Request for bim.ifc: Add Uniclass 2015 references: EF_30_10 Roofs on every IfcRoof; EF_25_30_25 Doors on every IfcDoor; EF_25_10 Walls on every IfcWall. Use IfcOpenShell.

First a look at what the model holds.

```python
import ifcopenshell

model = ifcopenshell.open("bim.ifc")
print(model.schema)
print("classifications:", [c.Name for c in model.by_type("IfcClassification")])
for ifc_class in ("IfcDoor", "IfcRoof", "IfcStair", "IfcWall", "IfcWindow"):
    print(ifc_class, len(model.by_type(ifc_class)))
```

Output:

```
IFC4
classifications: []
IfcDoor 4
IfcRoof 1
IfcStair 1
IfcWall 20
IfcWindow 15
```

```python
import ifcopenshell
import ifcopenshell.api.classification

model = ifcopenshell.open("bim.ifc")

system = ifcopenshell.api.classification.add_classification(model, classification="Uniclass 2015")

codes = {
    "IfcRoof": ("EF_30_10", "Roofs"),
    "IfcDoor": ("EF_25_30_25", "Doors"),
    "IfcWall": ("EF_25_10", "Walls"),
}
for ifc_class, (code, name) in codes.items():
    products = model.by_type(ifc_class)
    ifcopenshell.api.classification.add_reference(
        model, products=products, classification=system, identification=code, name=name
    )
    print(code, len(products))

model.write("bim_edited.ifc")
```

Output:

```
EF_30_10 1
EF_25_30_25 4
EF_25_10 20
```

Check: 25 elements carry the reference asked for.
